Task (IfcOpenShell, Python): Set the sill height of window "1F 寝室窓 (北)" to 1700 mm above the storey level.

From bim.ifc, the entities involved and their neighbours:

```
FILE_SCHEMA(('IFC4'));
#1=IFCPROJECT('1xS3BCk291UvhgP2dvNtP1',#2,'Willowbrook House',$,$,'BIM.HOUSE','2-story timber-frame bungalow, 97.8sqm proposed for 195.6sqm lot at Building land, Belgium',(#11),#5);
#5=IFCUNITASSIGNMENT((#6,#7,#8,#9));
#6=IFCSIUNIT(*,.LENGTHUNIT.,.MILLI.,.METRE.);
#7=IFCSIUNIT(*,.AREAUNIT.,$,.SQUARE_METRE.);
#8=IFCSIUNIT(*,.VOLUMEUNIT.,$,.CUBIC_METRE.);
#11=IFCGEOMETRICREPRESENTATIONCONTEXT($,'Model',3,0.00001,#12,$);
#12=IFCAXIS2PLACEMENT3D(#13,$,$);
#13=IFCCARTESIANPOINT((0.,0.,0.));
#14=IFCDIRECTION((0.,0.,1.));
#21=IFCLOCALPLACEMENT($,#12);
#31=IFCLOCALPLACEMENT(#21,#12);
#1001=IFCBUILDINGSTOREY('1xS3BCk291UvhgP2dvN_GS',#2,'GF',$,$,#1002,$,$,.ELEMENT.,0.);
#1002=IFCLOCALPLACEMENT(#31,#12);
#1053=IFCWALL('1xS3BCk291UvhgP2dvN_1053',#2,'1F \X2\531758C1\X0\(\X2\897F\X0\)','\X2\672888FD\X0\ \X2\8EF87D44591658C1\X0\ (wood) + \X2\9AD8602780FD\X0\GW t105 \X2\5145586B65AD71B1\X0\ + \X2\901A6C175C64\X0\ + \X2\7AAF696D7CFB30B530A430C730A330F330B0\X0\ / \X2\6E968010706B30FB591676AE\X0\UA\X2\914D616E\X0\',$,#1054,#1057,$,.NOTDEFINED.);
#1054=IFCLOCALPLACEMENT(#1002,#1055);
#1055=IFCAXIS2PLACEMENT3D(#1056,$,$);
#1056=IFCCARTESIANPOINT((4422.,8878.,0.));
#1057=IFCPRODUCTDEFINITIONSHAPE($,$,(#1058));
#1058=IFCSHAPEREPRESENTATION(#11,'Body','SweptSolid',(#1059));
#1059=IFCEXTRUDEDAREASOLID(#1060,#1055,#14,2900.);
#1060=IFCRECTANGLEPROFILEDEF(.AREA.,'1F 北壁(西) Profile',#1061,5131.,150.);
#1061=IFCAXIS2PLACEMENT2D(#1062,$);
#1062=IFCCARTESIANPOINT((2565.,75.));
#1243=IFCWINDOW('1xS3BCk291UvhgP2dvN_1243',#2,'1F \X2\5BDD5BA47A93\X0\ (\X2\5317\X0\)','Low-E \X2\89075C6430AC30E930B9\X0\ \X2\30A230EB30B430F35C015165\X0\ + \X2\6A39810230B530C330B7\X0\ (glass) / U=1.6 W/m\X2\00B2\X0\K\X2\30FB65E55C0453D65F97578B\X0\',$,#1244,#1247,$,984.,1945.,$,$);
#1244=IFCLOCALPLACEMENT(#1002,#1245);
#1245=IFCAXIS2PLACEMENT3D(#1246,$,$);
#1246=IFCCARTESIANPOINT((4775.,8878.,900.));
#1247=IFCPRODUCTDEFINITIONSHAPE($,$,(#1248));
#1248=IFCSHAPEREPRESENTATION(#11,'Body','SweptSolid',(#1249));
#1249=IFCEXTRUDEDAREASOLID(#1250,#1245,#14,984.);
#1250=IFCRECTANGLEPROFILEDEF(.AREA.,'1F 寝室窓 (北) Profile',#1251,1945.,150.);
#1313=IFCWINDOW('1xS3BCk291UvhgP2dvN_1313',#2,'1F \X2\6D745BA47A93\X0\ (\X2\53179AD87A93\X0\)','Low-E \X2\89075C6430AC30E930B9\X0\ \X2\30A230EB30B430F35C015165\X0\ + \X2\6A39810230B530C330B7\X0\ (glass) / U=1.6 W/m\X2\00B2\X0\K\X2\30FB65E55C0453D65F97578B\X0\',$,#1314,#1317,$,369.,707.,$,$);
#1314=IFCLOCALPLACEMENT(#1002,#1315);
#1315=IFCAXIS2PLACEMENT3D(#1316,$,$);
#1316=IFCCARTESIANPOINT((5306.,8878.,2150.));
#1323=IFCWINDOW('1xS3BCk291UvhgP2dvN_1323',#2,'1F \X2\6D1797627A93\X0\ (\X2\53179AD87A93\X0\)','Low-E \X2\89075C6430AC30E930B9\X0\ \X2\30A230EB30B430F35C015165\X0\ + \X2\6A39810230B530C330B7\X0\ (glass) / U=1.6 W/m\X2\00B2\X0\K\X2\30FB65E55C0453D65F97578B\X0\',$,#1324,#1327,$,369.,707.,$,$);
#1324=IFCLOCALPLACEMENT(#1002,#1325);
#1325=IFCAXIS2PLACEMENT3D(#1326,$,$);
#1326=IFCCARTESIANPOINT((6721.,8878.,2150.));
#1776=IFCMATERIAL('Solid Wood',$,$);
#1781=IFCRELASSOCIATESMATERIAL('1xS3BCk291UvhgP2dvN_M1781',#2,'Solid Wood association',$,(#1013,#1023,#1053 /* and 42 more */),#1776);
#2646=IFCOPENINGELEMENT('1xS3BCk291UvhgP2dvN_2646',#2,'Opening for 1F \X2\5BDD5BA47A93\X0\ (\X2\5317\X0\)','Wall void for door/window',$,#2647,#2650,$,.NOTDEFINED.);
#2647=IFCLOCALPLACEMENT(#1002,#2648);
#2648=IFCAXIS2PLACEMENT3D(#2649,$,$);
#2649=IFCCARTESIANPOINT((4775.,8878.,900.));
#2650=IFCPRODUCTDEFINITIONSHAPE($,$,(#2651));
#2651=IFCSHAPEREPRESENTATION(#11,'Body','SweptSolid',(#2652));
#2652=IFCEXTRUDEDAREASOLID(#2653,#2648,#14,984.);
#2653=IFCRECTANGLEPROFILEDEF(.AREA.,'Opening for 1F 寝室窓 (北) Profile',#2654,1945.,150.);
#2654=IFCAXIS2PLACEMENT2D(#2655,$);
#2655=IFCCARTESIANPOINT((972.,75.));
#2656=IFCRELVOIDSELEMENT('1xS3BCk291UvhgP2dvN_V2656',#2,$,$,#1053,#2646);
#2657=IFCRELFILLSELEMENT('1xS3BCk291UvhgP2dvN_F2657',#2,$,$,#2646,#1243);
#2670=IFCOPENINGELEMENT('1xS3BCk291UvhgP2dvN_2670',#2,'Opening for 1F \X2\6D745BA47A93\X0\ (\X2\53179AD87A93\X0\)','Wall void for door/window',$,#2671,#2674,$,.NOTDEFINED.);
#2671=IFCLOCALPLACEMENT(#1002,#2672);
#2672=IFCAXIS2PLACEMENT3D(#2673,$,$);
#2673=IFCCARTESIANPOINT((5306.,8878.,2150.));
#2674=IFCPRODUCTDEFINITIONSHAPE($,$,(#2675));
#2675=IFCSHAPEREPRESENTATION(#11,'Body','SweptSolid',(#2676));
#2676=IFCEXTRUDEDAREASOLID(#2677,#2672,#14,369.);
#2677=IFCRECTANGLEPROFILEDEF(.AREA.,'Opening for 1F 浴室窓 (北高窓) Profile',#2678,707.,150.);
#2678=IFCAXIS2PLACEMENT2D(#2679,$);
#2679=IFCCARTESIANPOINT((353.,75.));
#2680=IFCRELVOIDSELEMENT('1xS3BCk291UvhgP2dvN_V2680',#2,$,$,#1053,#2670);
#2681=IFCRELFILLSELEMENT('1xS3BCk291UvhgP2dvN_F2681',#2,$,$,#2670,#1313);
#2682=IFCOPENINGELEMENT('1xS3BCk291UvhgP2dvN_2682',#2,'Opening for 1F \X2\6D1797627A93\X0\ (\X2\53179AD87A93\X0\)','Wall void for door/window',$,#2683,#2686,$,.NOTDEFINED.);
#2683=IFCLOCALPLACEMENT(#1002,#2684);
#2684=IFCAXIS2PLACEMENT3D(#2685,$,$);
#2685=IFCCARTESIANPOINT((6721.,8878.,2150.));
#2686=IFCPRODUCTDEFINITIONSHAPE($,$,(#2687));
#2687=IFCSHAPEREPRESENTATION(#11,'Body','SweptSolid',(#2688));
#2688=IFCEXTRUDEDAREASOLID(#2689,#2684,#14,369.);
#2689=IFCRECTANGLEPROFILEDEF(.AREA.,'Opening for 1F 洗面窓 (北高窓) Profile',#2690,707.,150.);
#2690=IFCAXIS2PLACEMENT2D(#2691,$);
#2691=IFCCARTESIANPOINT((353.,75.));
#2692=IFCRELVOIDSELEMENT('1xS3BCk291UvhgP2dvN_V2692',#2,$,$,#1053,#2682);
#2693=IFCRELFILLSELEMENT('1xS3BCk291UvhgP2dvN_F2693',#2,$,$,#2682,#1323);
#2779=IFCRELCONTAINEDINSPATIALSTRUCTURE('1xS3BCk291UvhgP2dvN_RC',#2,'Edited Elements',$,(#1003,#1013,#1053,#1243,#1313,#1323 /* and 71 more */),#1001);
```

```python
import numpy as np
import ifcopenshell
import ifcopenshell.api.geometry
import ifcopenshell.geom
import ifcopenshell.util.element
import ifcopenshell.util.placement
import ifcopenshell.util.shape
import ifcopenshell.util.unit

model = ifcopenshell.open("bim.ifc")
unit_scale = ifcopenshell.util.unit.calculate_unit_scale(model)

window = model.by_guid("1xS3BCk291UvhgP2dvN_1243")
opening = window.FillsVoids[0].RelatingOpeningElement
storey = ifcopenshell.util.element.get_container(window, ifc_class="IfcBuildingStorey")
level = ifcopenshell.util.placement.get_local_placement(storey.ObjectPlacement)[2, 3]

# The opening's origin need not be at the sill, so measure its lowest point.
shape = ifcopenshell.geom.create_shape(ifcopenshell.geom.settings(), opening)
bottom = ifcopenshell.util.shape.get_shape_bottom_elevation(shape, shape.geometry) / unit_scale
dz = level + 1700.0 - bottom

shift = np.array([0.0, 0.0, dz])
# The window is not placed relative to its opening, so move both.
for product in (opening, window):
    matrix = ifcopenshell.util.placement.get_local_placement(product.ObjectPlacement)
    matrix[:3, 3] += shift
    ifcopenshell.api.geometry.edit_object_placement(model, product=product, matrix=matrix, is_si=False)

print(f"moved by {dz * unit_scale:+.3f} m")

model.write("bim-out.ifc")
```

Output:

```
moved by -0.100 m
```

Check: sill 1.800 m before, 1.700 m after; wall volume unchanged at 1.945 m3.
